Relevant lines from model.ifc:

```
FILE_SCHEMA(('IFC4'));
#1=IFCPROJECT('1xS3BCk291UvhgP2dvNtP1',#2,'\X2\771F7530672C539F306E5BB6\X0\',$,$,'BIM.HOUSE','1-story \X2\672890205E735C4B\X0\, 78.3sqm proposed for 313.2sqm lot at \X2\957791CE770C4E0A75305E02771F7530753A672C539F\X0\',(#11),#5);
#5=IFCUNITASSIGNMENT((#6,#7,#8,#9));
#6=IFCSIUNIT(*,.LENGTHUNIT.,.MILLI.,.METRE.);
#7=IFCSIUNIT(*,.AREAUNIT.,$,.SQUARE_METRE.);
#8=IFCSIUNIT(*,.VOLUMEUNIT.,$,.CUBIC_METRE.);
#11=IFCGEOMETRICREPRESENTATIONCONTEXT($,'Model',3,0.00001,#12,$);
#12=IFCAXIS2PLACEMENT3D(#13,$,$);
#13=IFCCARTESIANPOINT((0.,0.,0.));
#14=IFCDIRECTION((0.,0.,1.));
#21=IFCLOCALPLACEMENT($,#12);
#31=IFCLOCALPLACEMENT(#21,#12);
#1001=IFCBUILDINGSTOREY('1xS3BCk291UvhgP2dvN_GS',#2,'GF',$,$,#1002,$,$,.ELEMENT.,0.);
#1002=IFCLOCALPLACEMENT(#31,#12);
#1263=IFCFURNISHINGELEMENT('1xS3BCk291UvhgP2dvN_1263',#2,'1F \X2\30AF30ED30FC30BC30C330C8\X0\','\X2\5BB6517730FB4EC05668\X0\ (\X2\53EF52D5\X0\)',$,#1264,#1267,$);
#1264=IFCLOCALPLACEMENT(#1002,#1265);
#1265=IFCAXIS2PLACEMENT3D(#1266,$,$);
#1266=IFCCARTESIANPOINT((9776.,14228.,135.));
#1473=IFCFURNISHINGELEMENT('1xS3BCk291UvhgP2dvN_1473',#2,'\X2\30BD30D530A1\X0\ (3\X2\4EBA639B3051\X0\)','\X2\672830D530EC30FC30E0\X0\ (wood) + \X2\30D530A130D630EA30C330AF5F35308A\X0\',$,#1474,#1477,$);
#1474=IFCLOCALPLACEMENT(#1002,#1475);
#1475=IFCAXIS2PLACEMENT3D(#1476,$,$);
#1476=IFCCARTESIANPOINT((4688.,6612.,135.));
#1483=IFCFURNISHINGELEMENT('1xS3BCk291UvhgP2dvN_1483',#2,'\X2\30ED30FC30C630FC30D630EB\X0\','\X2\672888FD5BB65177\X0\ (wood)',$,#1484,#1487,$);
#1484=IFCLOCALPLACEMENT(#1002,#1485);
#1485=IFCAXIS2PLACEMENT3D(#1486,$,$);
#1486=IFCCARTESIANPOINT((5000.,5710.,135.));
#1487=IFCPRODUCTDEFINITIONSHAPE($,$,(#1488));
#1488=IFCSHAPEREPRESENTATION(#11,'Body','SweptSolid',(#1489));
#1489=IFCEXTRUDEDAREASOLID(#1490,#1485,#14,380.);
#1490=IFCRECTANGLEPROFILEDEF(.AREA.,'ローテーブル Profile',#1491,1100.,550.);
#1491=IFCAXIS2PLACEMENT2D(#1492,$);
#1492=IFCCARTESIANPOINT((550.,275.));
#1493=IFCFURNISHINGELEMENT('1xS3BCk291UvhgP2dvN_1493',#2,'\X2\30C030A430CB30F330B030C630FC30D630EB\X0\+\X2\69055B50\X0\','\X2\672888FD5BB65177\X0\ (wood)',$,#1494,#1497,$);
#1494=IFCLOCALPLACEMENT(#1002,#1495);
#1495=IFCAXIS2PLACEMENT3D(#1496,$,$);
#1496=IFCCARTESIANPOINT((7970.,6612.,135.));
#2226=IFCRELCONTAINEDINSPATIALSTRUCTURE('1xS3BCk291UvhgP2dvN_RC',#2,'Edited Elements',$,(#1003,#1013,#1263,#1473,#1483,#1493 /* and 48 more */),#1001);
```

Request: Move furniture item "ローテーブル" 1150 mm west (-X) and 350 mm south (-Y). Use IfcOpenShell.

```python
import ifcopenshell
import ifcopenshell.api.geometry
import ifcopenshell.util.placement
import ifcopenshell.util.unit

model = ifcopenshell.open("model.ifc")
unit_scale = ifcopenshell.util.unit.calculate_unit_scale(model)

item = model.by_guid("1xS3BCk291UvhgP2dvN_1483")
matrix = ifcopenshell.util.placement.get_local_placement(item.ObjectPlacement)
matrix[0, 3] -= 1.15 / unit_scale
matrix[1, 3] -= 0.35 / unit_scale
ifcopenshell.api.geometry.edit_object_placement(model, product=item, matrix=matrix, is_si=False)

print(ifcopenshell.util.placement.get_local_placement(item.ObjectPlacement).round(3) + 0.0)

model.write("model-out.ifc")
```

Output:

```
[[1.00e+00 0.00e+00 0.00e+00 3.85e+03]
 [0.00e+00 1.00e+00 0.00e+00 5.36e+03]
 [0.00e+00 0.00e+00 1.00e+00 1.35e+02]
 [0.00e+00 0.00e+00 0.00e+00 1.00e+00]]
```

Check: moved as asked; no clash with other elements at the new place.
